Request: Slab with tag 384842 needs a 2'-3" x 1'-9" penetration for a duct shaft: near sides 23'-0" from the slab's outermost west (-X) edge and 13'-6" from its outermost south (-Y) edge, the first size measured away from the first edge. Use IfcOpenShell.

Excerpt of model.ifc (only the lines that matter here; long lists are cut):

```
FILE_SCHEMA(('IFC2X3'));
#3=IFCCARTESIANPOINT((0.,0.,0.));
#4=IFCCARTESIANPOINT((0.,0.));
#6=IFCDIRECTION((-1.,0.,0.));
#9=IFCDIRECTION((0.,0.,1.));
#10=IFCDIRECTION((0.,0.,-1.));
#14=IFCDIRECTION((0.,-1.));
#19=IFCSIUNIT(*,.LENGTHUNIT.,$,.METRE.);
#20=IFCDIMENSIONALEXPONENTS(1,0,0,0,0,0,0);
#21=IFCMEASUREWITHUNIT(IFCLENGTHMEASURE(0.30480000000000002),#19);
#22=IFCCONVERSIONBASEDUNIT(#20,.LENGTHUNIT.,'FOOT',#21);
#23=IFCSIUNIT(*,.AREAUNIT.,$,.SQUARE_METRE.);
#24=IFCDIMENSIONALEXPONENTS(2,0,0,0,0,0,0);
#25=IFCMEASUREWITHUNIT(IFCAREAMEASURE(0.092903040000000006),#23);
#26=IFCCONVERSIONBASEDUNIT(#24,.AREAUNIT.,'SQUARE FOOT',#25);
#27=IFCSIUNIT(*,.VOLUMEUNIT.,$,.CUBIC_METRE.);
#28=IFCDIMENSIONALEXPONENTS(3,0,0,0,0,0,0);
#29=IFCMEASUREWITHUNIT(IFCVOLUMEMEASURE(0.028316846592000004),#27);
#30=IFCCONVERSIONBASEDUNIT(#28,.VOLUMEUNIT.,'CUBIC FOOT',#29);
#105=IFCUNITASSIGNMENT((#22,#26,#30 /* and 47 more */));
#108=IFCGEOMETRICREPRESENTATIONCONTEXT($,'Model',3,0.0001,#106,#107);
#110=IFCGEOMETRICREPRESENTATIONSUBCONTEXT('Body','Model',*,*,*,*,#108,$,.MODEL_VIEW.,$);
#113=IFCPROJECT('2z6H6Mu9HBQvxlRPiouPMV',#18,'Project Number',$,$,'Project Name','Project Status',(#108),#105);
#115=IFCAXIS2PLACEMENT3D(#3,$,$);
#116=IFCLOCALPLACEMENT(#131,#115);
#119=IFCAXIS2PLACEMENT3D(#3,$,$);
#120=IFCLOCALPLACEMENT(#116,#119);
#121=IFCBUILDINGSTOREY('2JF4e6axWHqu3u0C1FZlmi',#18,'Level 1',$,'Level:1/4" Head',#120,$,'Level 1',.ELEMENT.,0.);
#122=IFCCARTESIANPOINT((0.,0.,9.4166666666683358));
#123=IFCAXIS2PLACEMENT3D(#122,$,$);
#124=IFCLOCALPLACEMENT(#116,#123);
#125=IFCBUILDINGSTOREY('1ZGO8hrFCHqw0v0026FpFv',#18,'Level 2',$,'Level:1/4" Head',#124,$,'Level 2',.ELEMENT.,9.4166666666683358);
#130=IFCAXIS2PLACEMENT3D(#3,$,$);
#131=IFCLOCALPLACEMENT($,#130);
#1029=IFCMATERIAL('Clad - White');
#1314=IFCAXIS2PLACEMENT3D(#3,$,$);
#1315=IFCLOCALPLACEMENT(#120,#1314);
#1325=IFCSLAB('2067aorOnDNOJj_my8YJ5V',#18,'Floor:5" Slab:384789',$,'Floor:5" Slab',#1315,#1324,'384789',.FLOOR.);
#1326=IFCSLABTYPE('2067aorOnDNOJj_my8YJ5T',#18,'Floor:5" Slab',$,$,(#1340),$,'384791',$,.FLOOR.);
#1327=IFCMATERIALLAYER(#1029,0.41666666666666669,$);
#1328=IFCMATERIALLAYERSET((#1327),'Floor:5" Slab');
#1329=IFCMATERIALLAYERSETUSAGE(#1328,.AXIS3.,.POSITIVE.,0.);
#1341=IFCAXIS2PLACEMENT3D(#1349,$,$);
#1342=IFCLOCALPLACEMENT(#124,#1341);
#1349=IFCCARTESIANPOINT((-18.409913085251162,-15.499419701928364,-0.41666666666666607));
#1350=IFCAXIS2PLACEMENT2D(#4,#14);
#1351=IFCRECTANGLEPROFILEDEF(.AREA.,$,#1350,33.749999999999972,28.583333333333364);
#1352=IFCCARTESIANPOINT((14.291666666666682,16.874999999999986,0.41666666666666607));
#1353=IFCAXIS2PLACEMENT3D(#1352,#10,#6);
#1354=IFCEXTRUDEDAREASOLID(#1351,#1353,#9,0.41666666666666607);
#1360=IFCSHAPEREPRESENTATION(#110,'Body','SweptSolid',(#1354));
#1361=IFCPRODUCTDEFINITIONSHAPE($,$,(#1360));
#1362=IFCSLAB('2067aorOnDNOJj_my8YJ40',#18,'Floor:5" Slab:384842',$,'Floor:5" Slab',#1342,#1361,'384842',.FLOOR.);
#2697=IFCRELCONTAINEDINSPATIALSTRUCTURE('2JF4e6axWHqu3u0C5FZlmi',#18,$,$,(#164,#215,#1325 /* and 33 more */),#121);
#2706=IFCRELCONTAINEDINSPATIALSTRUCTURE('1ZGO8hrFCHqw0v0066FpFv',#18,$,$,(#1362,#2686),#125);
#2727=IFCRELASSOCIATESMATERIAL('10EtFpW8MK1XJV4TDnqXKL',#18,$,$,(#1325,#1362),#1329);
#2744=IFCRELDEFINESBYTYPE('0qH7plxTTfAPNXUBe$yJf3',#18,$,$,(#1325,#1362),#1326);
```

```python
import numpy as np
import ifcopenshell
import ifcopenshell.api.feature
import ifcopenshell.api.geometry
import ifcopenshell.api.root
import ifcopenshell.geom
import ifcopenshell.util.placement
import ifcopenshell.util.representation
import ifcopenshell.util.shape
import ifcopenshell.util.unit

model = ifcopenshell.open("model.ifc")
unit_scale = ifcopenshell.util.unit.calculate_unit_scale(model)
settings = ifcopenshell.geom.settings()


def volume(element):
    """Net volume in cubic metres, openings subtracted."""
    shape = ifcopenshell.geom.create_shape(settings, element)
    return ifcopenshell.util.shape.get_volume(shape.geometry)


slab = model.by_id(1362)
before = volume(slab)

# Extent in the slab's own axes, in metres. The edges named are its -X and -Y sides.
slab_shape = ifcopenshell.geom.create_shape(settings, slab)
vertices = ifcopenshell.util.shape.get_vertices(slab_shape.geometry)
x_min, y_min, bottom = vertices.min(axis=0)
top = vertices[:, 2].max()

opening = ifcopenshell.api.root.create_entity(model, ifc_class="IfcOpeningElement", name="Duct shaft opening")
context = ifcopenshell.util.representation.get_context(model, "Model", "Body", "MODEL_VIEW")
width, depth = 0.6858, 0.5334
outline = [(0.0, 0.0), (width, 0.0), (width, depth), (0.0, depth), (0.0, 0.0)]
# Overshoot both faces by 50 mm so the cut is clean.
shape = ifcopenshell.api.geometry.add_slab_representation(
    model, context=context, depth=top - bottom + 0.1, polyline=outline
)
ifcopenshell.api.geometry.assign_representation(model, product=opening, representation=shape)

matrix = ifcopenshell.util.placement.get_local_placement(slab.ObjectPlacement)
matrix[:, 3] = matrix @ np.append(np.array([x_min + 7.0104, y_min + 4.1148, bottom - 0.05]) / unit_scale, 1.0)
ifcopenshell.api.geometry.edit_object_placement(model, product=opening, matrix=matrix, is_si=False)
ifcopenshell.api.feature.add_feature(model, feature=opening, element=slab)

after = volume(slab)

print(f"slab volume {before:.3f} -> {after:.3f} m3")

model.write("model_edited.ifc")
```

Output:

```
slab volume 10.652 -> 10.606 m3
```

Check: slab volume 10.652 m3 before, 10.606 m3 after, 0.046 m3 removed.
